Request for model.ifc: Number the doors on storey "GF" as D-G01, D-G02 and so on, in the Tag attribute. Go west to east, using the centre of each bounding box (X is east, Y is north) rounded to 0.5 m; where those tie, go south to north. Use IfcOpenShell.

First a look at what the model holds.

```python
import ifcopenshell
import ifcopenshell.util.element
import ifcopenshell.util.placement

model = ifcopenshell.open("model.ifc")
print(model.schema)
storey = next(s for s in model.by_type("IfcBuildingStorey") if s.Name == "GF")
doors = [e for e in ifcopenshell.util.element.get_decomposition(storey) if e.is_a("IfcDoor")]
for e in sorted(doors, key=lambda e: e.id()):
    origin = ifcopenshell.util.placement.get_local_placement(e.ObjectPlacement)[:3, 3]
    print(e.id(), e.Tag, e.Name, origin.round(2) + 0.0, sep=" | ")
```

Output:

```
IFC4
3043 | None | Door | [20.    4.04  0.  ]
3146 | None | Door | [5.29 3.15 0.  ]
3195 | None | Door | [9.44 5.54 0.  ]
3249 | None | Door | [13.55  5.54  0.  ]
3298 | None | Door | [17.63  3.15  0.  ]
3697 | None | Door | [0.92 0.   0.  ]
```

```python
import ifcopenshell
import ifcopenshell.geom
import ifcopenshell.util.element
import ifcopenshell.util.shape

model = ifcopenshell.open("model.ifc")
settings = ifcopenshell.geom.settings()
settings.set("use-world-coords", True)


def centre(element):
    shape = ifcopenshell.geom.create_shape(settings, element)
    return ifcopenshell.util.shape.get_bbox_centroid(shape.geometry)


storey = next(s for s in model.by_type("IfcBuildingStorey") if s.Name == "GF")
doors = [e for e in ifcopenshell.util.element.get_decomposition(storey) if e.is_a("IfcDoor")]

# Insertion points can sit at a corner or the storey origin, so sort by the geometry (in metres).
centres = {e: centre(e) for e in doors}
doors.sort(key=lambda e: (round(centres[e][0] / 0.5), centres[e][1]))

for i, e in enumerate(doors, start=1):
    number = f"D-G{i:02d}"
    e.Tag = number
    print(e.id(), number)

model.write("model_rev.ifc")
```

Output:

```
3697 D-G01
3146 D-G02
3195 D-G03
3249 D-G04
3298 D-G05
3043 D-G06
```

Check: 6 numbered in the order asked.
